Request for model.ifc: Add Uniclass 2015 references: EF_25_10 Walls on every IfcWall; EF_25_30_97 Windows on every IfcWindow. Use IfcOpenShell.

First a look at what the model holds.

```python
import ifcopenshell

model = ifcopenshell.open("model.ifc")
print(model.schema)
print("classifications:", [c.Name for c in model.by_type("IfcClassification")])
for ifc_class in ("IfcDoor", "IfcRoof", "IfcStair", "IfcWall", "IfcWindow"):
    print(ifc_class, len(model.by_type(ifc_class)))
```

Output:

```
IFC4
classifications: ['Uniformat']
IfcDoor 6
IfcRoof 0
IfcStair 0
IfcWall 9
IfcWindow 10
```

```python
import ifcopenshell
import ifcopenshell.api.classification

model = ifcopenshell.open("model.ifc")

system = ifcopenshell.api.classification.add_classification(model, classification="Uniclass 2015")

codes = {
    "IfcWall": ("EF_25_10", "Walls"),
    "IfcWindow": ("EF_25_30_97", "Windows"),
}
for ifc_class, (code, name) in codes.items():
    products = model.by_type(ifc_class)
    ifcopenshell.api.classification.add_reference(
        model, products=products, classification=system, identification=code, name=name
    )
    print(code, len(products))

model.write("model_rev.ifc")
```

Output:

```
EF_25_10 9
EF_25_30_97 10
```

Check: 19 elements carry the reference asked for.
